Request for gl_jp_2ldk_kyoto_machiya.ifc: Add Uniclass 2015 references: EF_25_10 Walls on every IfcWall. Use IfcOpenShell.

First a look at what the model holds.

```python
import ifcopenshell

model = ifcopenshell.open("gl_jp_2ldk_kyoto_machiya.ifc")
print(model.schema)
print("classifications:", [c.Name for c in model.by_type("IfcClassification")])
for ifc_class in ("IfcDoor", "IfcRoof", "IfcStair", "IfcWall", "IfcWindow"):
    print(ifc_class, len(model.by_type(ifc_class)))
```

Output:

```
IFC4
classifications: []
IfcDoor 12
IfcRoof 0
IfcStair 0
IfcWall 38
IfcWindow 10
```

```python
import ifcopenshell
import ifcopenshell.api.classification

model = ifcopenshell.open("gl_jp_2ldk_kyoto_machiya.ifc")

system = ifcopenshell.api.classification.add_classification(model, classification="Uniclass 2015")

codes = {
    "IfcWall": ("EF_25_10", "Walls"),
}
for ifc_class, (code, name) in codes.items():
    products = model.by_type(ifc_class)
    ifcopenshell.api.classification.add_reference(
        model, products=products, classification=system, identification=code, name=name
    )
    print(code, len(products))

model.write("gl_jp_2ldk_kyoto_machiya-out.ifc")
```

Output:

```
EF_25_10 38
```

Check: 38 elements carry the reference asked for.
